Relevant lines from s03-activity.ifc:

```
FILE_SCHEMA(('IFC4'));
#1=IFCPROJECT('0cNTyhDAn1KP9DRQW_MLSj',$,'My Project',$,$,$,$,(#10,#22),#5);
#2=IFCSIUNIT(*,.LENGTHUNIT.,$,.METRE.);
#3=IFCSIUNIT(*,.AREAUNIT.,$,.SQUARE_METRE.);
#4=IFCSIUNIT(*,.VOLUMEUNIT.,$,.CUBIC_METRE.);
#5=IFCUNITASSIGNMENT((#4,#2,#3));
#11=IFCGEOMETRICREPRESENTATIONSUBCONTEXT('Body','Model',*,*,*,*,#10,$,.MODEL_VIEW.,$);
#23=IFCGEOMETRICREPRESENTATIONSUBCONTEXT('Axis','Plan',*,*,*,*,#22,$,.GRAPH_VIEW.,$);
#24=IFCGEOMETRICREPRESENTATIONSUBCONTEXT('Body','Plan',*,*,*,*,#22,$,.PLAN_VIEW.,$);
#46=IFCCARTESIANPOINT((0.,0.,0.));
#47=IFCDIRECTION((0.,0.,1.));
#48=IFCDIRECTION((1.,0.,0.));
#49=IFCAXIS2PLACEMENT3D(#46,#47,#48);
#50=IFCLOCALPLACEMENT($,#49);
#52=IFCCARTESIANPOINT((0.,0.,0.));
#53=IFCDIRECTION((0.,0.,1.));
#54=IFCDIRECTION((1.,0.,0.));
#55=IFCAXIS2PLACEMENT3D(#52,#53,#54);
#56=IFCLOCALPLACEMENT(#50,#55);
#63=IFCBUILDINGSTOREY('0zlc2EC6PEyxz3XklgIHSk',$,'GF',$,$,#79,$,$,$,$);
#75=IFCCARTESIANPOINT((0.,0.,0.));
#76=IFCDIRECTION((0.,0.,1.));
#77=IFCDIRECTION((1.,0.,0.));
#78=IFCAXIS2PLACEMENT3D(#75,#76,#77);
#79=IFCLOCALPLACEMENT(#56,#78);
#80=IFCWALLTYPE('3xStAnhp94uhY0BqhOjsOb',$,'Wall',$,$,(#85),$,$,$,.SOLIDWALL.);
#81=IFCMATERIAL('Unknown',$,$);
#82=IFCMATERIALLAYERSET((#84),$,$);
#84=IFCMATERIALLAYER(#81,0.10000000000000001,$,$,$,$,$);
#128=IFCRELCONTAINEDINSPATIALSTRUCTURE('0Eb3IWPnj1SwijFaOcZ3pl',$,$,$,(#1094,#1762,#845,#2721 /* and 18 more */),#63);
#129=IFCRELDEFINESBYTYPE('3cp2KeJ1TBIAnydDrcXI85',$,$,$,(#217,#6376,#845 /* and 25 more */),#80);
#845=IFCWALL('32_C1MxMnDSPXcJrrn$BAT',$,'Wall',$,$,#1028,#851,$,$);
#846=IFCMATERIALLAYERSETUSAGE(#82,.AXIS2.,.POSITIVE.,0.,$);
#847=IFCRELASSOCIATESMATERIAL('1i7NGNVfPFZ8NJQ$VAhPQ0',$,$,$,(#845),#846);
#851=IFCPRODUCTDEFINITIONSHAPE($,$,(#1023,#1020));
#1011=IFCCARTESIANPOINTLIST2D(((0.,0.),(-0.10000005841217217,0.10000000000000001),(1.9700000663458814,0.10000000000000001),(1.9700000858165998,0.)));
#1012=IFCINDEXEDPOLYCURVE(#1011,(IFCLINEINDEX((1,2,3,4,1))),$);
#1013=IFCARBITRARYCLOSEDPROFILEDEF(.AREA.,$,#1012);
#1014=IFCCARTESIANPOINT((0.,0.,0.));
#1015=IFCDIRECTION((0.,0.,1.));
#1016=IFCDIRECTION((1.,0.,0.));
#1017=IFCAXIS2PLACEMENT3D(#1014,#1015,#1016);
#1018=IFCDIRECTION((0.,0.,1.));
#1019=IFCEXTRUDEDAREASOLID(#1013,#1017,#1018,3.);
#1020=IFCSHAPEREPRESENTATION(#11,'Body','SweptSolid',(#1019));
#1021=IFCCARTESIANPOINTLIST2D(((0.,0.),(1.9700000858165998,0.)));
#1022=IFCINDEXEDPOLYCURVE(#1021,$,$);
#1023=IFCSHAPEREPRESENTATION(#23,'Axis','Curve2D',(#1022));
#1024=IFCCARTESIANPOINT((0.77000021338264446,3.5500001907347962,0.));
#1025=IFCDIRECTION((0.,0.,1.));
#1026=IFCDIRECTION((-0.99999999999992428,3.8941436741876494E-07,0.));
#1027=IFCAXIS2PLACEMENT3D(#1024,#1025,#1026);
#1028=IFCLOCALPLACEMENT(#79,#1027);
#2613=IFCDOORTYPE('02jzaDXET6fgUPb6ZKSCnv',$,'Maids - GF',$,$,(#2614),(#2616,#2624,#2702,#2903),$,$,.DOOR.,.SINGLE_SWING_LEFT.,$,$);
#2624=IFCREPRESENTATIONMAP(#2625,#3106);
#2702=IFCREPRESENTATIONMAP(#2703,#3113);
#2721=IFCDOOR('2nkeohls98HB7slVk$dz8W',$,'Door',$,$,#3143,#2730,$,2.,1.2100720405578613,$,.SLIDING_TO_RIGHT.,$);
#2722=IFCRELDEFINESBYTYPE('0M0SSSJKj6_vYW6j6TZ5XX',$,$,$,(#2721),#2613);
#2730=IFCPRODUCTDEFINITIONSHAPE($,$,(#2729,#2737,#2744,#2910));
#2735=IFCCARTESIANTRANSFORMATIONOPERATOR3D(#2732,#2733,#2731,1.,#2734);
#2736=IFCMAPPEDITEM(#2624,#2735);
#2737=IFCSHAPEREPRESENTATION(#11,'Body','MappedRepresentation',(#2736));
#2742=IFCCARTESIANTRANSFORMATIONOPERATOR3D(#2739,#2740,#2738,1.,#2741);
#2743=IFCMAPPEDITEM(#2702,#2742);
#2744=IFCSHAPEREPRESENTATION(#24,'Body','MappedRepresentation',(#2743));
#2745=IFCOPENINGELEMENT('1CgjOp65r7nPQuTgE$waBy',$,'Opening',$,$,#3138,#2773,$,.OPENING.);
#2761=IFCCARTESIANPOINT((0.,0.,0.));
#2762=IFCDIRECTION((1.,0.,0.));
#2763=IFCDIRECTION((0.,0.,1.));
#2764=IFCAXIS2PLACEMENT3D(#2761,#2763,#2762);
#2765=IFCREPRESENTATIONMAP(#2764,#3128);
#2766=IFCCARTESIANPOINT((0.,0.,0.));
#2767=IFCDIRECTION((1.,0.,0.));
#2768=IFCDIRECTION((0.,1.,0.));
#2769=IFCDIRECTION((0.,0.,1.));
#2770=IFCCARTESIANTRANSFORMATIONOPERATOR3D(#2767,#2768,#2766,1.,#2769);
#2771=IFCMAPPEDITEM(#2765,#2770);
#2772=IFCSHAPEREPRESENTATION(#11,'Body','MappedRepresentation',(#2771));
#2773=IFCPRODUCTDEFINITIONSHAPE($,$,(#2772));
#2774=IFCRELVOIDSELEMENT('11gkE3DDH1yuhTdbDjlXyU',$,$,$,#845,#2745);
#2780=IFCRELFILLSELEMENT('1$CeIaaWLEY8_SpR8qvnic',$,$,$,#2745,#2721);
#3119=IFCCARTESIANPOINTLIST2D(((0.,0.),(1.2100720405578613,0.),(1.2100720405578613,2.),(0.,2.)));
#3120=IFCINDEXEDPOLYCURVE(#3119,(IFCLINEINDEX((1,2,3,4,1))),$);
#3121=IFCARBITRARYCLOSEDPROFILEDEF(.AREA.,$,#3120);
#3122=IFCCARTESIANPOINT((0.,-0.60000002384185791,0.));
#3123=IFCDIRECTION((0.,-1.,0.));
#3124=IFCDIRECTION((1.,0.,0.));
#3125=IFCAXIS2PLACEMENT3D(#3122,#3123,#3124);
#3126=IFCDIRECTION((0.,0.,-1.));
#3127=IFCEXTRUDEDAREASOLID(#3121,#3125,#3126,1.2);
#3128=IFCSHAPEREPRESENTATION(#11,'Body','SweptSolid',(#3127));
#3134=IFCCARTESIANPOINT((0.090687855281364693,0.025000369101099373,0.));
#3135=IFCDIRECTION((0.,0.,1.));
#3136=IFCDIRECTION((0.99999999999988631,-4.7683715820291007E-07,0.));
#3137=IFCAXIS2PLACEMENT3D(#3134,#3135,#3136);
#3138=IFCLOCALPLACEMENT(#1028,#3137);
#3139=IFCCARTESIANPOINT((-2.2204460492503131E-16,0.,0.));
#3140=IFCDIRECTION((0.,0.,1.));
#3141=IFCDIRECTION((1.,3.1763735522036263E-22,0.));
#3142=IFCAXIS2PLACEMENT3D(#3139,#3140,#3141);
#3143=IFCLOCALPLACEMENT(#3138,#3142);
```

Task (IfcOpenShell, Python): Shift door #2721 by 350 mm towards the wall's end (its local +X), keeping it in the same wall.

```python
import ifcopenshell
import ifcopenshell.api.geometry
import ifcopenshell.util.placement
import ifcopenshell.util.unit

model = ifcopenshell.open("s03-activity.ifc")
unit_scale = ifcopenshell.util.unit.calculate_unit_scale(model)

door = model.by_id(2721)
opening = door.FillsVoids[0].RelatingOpeningElement
wall = opening.VoidsElements[0].RelatingBuildingElement

wall_matrix = ifcopenshell.util.placement.get_local_placement(wall.ObjectPlacement)
shift = wall_matrix[:3, 0] * 0.35 / unit_scale
before = ifcopenshell.util.placement.get_local_placement(door.ObjectPlacement)[:3, 3].copy()

# The door is placed relative to its opening, so it follows when the opening moves.
matrix = ifcopenshell.util.placement.get_local_placement(opening.ObjectPlacement)
matrix[:3, 3] += shift
ifcopenshell.api.geometry.edit_object_placement(
    model, product=opening, matrix=matrix, is_si=False, should_transform_children=True
)

after = ifcopenshell.util.placement.get_local_placement(door.ObjectPlacement)[:3, 3]
print("door moved by", (after - before).round(3) + 0.0)

model.write("s03-activity_updated.ifc")
```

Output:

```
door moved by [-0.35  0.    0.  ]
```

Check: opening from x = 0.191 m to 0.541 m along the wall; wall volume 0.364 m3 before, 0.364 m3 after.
